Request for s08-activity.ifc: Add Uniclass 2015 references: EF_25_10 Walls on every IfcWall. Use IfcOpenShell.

First a look at what the model holds.

```python
import ifcopenshell

model = ifcopenshell.open("s08-activity.ifc")
print(model.schema)
print("classifications:", [c.Name for c in model.by_type("IfcClassification")])
for ifc_class in ("IfcDoor", "IfcRoof", "IfcStair", "IfcWall", "IfcWindow"):
    print(ifc_class, len(model.by_type(ifc_class)))
```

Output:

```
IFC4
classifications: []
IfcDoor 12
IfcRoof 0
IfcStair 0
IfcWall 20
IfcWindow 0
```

```python
import ifcopenshell
import ifcopenshell.api.classification

model = ifcopenshell.open("s08-activity.ifc")

system = ifcopenshell.api.classification.add_classification(model, classification="Uniclass 2015")

codes = {
    "IfcWall": ("EF_25_10", "Walls"),
}
for ifc_class, (code, name) in codes.items():
    products = model.by_type(ifc_class)
    ifcopenshell.api.classification.add_reference(
        model, products=products, classification=system, identification=code, name=name
    )
    print(code, len(products))

model.write("s08-activity_rev.ifc")
```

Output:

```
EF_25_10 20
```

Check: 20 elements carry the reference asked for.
